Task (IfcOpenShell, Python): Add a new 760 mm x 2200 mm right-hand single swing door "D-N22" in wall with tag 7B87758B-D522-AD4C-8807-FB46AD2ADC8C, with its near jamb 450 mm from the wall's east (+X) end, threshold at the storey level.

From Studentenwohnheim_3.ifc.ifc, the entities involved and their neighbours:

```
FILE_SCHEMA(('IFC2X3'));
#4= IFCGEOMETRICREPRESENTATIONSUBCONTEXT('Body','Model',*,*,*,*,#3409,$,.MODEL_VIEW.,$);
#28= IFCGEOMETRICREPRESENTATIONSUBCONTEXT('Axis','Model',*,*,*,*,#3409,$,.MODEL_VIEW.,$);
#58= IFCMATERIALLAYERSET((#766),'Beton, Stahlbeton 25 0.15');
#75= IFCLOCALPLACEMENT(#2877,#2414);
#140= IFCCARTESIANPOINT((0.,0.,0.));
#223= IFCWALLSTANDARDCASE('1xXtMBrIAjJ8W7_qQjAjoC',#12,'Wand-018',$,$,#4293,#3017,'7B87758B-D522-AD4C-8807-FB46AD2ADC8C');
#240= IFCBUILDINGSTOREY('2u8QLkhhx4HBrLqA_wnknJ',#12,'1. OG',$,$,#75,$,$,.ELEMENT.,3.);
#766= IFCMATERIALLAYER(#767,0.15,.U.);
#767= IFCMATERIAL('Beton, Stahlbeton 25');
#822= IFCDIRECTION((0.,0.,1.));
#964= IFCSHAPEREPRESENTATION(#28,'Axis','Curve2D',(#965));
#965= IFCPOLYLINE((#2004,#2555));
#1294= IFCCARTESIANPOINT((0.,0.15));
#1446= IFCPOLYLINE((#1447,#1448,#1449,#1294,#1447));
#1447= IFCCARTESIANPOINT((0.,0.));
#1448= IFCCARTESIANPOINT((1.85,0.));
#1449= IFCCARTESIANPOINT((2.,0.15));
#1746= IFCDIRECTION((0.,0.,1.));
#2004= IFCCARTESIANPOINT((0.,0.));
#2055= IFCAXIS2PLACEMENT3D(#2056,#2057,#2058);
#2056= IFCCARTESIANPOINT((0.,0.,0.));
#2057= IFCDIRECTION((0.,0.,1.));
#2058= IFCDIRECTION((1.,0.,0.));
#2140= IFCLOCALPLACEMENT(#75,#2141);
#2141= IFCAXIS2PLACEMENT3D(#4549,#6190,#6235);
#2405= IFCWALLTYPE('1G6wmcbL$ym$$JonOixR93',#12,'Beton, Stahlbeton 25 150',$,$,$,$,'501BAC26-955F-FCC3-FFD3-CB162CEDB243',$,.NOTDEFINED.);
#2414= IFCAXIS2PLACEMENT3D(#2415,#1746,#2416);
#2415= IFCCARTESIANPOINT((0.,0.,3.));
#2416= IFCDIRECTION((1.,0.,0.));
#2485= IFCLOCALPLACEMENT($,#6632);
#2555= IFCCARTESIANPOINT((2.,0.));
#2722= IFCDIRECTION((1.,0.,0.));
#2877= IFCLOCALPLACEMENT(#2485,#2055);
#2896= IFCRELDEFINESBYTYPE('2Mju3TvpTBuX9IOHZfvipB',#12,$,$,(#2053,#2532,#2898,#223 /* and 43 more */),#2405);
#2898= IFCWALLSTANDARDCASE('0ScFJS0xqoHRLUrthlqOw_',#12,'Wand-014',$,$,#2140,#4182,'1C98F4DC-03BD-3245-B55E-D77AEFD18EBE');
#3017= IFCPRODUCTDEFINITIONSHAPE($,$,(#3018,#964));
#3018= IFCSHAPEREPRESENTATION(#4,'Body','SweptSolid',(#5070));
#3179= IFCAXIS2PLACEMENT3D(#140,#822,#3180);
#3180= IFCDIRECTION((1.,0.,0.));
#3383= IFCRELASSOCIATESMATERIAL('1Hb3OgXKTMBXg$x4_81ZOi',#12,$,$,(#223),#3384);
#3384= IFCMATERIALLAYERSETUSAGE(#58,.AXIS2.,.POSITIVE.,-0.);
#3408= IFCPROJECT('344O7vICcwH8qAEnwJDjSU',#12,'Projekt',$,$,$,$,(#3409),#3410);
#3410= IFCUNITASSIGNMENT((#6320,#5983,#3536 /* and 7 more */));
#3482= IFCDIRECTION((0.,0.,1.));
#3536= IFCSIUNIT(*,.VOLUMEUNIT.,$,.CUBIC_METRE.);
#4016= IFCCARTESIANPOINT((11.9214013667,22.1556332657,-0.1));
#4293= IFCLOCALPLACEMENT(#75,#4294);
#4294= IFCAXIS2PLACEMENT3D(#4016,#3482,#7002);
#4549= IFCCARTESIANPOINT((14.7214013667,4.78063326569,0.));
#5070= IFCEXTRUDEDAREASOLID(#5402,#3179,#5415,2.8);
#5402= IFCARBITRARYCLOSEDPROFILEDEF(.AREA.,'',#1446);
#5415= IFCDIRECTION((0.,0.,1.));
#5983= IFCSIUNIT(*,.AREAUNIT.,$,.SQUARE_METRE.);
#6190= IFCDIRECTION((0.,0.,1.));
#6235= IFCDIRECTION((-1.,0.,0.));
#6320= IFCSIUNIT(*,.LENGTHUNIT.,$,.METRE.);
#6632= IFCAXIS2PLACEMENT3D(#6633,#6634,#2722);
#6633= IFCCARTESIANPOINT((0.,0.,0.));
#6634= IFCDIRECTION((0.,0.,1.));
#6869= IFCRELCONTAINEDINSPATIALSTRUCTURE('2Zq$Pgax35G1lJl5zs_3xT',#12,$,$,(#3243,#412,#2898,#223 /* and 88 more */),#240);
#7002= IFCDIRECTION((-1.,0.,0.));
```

```python
import numpy as np
import ifcopenshell
import ifcopenshell.api.feature
import ifcopenshell.api.geometry
import ifcopenshell.api.root
import ifcopenshell.api.spatial
import ifcopenshell.api.type
import ifcopenshell.geom
import ifcopenshell.util.element
import ifcopenshell.util.placement
import ifcopenshell.util.representation
import ifcopenshell.util.shape
import ifcopenshell.util.unit

model = ifcopenshell.open("Studentenwohnheim_3.ifc.ifc")
unit_scale = ifcopenshell.util.unit.calculate_unit_scale(model)
settings = ifcopenshell.geom.settings()


def volume(element):
    """Net volume in cubic metres, openings subtracted."""
    shape = ifcopenshell.geom.create_shape(settings, element)
    return ifcopenshell.util.shape.get_volume(shape.geometry)


wall = model.by_guid("1xXtMBrIAjJ8W7_qQjAjoC")
storey = ifcopenshell.util.element.get_container(wall, ifc_class="IfcBuildingStorey")
context = ifcopenshell.util.representation.get_context(model, "Model", "Body", "MODEL_VIEW")
before = volume(wall)

width, height, from_end, sill = 0.76, 2.2, 0.45, 0.0  # metres

# The wall runs along its own X axis, and the end named is its -X end.
wall_shape = ifcopenshell.geom.create_shape(settings, wall)
x, y, z = ifcopenshell.util.shape.get_vertices(wall_shape.geometry).T
start = x.min() + from_end
face, thickness = float(y.min()), float(y.max() - y.min())
wall_matrix = ifcopenshell.util.placement.get_local_placement(wall.ObjectPlacement)
level = ifcopenshell.util.placement.get_local_placement(storey.ObjectPlacement)[2, 3]


def in_wall(x, y):
    """Placement at x, y metres in the wall's axes, at sill height."""
    matrix = wall_matrix.copy()
    matrix[:, 3] = wall_matrix @ np.array([x / unit_scale, y / unit_scale, 0.0, 1.0])
    matrix[2, 3] = level + sill / unit_scale
    return matrix


# Opening: a box that overshoots both wall faces by 50 mm.
opening = ifcopenshell.api.root.create_entity(model, ifc_class="IfcOpeningElement")
box = ifcopenshell.api.geometry.add_wall_representation(
    model, context=context, length=width, height=height, thickness=thickness + 0.1
)
ifcopenshell.api.geometry.assign_representation(model, product=opening, representation=box)
ifcopenshell.api.geometry.edit_object_placement(model, product=opening, matrix=in_wall(start, face - 0.05), is_si=False)
ifcopenshell.api.feature.add_feature(model, feature=opening, element=wall)

door = ifcopenshell.api.root.create_entity(model, ifc_class="IfcDoor", name="D-N22")
door.OverallWidth, door.OverallHeight = width / unit_scale, height / unit_scale
body = ifcopenshell.api.geometry.add_door_representation(
    model,
    context=context,
    overall_width=door.OverallWidth,
    overall_height=door.OverallHeight,
    operation_type="SINGLE_SWING_RIGHT",
    lining_properties={"LiningDepth": thickness / unit_scale, "ThresholdDepth": thickness / unit_scale},
)
ifcopenshell.api.geometry.assign_representation(model, product=door, representation=body)
ifcopenshell.api.spatial.assign_container(model, products=[door], relating_structure=storey)
fills = ifcopenshell.api.feature.add_filling(model, opening=opening, element=door)
fills.OwnerHistory = door.OwnerHistory  # required in IFC2X3

# IFC2X3 keeps the operation on the door style.
style = ifcopenshell.api.root.create_entity(model, ifc_class="IfcDoorStyle", name="D-N22")
style.OperationType, style.ConstructionType = "SINGLE_SWING_RIGHT", "NOTDEFINED"
style.ParameterTakesPrecedence = style.Sizeable = False
ifcopenshell.api.type.assign_type(model, related_objects=[door], relating_type=style)

# The lining spans the wall, so the door starts at the wall face.
ifcopenshell.api.geometry.edit_object_placement(model, product=door, matrix=in_wall(start, face), is_si=False)

after = volume(wall)

print(f"wall volume {before:.3f} -> {after:.3f} m3")

model.write("Studentenwohnheim_3.ifc_edited.ifc")
```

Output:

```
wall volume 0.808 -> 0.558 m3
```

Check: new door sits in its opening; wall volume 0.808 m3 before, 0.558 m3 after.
